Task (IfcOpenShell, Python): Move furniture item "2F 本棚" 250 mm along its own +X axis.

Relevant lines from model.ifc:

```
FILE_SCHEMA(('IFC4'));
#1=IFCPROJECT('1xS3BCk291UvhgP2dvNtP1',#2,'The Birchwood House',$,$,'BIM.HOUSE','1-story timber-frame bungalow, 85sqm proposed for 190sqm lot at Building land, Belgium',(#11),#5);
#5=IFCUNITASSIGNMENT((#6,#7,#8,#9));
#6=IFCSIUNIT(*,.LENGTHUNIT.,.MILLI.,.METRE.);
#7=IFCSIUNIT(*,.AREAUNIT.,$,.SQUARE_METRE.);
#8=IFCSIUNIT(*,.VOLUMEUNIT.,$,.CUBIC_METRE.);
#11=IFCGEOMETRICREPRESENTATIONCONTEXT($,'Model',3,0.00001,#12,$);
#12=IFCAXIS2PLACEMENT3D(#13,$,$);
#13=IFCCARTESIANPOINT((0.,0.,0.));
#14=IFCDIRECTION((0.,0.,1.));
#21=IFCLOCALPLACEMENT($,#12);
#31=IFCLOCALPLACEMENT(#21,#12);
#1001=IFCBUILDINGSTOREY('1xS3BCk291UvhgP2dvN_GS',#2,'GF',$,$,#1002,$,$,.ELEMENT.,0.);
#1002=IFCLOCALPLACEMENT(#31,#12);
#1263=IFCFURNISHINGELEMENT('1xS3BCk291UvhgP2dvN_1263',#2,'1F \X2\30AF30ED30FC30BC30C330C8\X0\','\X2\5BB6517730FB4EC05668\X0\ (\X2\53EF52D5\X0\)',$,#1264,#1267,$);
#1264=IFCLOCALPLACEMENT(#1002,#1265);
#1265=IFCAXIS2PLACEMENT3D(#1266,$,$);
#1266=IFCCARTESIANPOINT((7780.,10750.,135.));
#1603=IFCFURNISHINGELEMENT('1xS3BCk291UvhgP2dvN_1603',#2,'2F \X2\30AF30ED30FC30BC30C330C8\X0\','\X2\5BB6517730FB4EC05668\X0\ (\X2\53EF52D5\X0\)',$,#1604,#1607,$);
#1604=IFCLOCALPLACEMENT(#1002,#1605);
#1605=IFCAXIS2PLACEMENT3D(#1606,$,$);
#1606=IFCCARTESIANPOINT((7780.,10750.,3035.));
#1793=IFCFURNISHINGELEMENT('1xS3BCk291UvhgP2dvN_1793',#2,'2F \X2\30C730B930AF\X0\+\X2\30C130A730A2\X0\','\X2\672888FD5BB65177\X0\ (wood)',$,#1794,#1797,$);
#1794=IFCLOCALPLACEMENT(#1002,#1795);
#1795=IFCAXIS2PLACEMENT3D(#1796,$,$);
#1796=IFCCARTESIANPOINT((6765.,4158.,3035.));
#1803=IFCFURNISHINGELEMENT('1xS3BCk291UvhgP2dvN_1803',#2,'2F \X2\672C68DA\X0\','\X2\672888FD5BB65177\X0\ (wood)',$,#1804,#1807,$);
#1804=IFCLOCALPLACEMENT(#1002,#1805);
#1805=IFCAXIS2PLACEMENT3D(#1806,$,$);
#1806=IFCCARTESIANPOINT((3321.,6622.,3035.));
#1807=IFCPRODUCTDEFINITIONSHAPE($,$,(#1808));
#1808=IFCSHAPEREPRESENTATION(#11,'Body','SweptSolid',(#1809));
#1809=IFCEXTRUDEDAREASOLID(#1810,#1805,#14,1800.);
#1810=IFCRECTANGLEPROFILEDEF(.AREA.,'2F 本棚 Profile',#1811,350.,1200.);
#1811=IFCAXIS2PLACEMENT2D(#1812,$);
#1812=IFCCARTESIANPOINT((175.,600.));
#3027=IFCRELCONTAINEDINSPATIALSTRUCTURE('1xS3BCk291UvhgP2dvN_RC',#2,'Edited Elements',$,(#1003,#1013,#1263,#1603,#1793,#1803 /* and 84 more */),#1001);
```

```python
import ifcopenshell
import ifcopenshell.api.geometry
import ifcopenshell.util.placement
import ifcopenshell.util.unit

model = ifcopenshell.open("model.ifc")
unit_scale = ifcopenshell.util.unit.calculate_unit_scale(model)

item = model.by_guid("1xS3BCk291UvhgP2dvN_1803")
matrix = ifcopenshell.util.placement.get_local_placement(item.ObjectPlacement)
matrix[:3, 3] += matrix[:3, 0] * 0.25 / unit_scale
ifcopenshell.api.geometry.edit_object_placement(model, product=item, matrix=matrix, is_si=False)

print(ifcopenshell.util.placement.get_local_placement(item.ObjectPlacement).round(3) + 0.0)

model.write("model_rev.ifc")
```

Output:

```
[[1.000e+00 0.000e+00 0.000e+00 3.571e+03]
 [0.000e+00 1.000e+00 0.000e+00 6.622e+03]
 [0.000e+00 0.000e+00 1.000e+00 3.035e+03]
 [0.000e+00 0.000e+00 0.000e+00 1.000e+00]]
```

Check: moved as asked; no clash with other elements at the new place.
